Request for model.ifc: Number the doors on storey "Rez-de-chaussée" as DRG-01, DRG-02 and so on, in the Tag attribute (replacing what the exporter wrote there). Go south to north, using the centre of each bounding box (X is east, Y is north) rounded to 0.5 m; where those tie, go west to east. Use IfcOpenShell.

First a look at what the model holds.

```python
import ifcopenshell
import ifcopenshell.util.element
import ifcopenshell.util.placement

model = ifcopenshell.open("model.ifc")
print(model.schema)
storey = next(s for s in model.by_type("IfcBuildingStorey") if s.Name == "Rez-de-chaussée")
doors = [e for e in ifcopenshell.util.element.get_decomposition(storey) if e.is_a("IfcDoor")]
for e in sorted(doors, key=lambda e: e.id()):
    origin = ifcopenshell.util.placement.get_local_placement(e.ObjectPlacement)[:3, 3]
    print(e.id(), e.Tag, e.Name, origin.round(2) + 0.0, sep=" | ")
```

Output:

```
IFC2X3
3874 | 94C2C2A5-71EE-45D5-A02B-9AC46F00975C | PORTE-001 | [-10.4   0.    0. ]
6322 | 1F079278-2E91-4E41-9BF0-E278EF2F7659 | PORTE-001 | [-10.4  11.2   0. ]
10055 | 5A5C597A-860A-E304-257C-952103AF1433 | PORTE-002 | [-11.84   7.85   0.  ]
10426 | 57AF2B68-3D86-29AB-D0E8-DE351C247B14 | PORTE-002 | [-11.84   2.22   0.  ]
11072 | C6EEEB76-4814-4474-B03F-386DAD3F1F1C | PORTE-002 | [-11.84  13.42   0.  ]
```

```python
import ifcopenshell
import ifcopenshell.geom
import ifcopenshell.util.element
import ifcopenshell.util.shape

model = ifcopenshell.open("model.ifc")
settings = ifcopenshell.geom.settings()
settings.set("use-world-coords", True)


def centre(element):
    shape = ifcopenshell.geom.create_shape(settings, element)
    return ifcopenshell.util.shape.get_bbox_centroid(shape.geometry)


storey = next(s for s in model.by_type("IfcBuildingStorey") if s.Name == "Rez-de-chaussée")
doors = [e for e in ifcopenshell.util.element.get_decomposition(storey) if e.is_a("IfcDoor")]

# Insertion points can sit at a corner or the storey origin, so sort by the geometry (in metres).
centres = {e: centre(e) for e in doors}
doors.sort(key=lambda e: (round(centres[e][1] / 0.5), centres[e][0]))

for i, e in enumerate(doors, start=1):
    number = f"DRG-{i:02d}"
    e.Tag = number
    print(e.id(), number)

model.write("model-out.ifc")
```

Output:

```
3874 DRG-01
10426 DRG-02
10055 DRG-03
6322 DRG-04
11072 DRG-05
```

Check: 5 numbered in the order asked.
